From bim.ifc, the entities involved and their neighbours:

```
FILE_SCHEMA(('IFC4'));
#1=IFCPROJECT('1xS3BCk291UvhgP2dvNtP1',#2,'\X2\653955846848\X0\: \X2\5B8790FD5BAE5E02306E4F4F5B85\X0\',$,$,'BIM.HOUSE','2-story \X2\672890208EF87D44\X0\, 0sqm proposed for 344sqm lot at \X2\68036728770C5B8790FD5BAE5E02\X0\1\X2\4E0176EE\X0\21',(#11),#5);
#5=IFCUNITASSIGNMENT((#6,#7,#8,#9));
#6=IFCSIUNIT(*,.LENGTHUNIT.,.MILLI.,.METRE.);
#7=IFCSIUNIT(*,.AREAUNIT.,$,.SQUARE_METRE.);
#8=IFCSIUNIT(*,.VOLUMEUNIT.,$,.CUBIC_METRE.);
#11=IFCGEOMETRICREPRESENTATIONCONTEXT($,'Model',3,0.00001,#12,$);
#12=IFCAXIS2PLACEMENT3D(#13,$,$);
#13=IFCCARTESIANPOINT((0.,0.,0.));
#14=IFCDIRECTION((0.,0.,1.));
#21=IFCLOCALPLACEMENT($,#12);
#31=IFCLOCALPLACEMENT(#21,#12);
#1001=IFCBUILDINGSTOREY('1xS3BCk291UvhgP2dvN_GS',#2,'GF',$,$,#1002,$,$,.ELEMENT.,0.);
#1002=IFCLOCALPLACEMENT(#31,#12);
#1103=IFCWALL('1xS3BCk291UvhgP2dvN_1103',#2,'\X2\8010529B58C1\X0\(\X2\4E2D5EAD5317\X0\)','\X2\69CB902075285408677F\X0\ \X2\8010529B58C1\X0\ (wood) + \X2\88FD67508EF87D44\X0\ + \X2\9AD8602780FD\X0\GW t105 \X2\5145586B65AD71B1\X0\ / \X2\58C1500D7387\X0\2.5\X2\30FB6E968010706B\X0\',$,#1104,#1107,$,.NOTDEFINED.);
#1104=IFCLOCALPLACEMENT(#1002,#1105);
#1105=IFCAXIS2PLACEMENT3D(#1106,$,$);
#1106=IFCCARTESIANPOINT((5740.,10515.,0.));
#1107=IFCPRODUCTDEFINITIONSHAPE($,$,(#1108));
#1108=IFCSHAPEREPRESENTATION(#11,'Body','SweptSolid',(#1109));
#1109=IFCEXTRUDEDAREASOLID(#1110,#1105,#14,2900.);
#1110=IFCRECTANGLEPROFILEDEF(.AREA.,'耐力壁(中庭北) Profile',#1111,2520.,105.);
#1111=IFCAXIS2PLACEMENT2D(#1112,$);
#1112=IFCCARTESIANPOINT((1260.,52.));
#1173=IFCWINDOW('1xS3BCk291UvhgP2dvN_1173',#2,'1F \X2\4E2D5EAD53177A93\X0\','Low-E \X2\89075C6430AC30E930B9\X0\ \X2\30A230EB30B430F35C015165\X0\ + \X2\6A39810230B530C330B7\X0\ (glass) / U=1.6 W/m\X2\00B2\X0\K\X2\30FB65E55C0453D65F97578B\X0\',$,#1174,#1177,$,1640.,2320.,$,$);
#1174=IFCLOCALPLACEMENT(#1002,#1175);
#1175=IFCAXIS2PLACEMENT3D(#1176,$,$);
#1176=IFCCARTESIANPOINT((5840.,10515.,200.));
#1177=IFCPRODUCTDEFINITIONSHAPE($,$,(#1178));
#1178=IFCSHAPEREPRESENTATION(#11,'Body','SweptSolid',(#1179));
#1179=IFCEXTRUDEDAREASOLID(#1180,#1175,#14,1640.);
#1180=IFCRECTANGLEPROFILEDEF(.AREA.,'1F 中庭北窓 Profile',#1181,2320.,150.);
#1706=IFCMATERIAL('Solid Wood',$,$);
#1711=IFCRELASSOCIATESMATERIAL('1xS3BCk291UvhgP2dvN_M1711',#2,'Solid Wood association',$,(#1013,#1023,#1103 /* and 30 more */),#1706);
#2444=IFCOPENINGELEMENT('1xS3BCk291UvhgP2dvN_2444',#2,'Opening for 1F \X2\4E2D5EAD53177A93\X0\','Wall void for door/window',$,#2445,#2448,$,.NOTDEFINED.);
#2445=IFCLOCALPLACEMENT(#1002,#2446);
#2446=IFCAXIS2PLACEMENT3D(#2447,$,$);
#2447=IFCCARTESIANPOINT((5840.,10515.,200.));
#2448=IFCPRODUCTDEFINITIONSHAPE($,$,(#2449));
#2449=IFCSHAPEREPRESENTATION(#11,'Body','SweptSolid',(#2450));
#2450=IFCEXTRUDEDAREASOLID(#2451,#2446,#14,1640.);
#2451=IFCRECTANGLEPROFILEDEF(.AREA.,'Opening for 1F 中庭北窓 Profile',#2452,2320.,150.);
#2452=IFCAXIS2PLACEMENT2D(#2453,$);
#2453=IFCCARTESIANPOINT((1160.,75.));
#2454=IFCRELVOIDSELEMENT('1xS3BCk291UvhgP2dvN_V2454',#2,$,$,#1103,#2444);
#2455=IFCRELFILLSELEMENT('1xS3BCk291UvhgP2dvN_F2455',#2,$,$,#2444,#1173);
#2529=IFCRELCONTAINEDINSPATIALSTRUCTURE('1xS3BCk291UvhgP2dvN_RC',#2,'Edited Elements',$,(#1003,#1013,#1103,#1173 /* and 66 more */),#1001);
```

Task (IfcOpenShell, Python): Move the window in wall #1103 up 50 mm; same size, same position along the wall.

```python
import numpy as np
import ifcopenshell
import ifcopenshell.api.geometry
import ifcopenshell.util.placement
import ifcopenshell.util.unit

model = ifcopenshell.open("bim.ifc")
unit_scale = ifcopenshell.util.unit.calculate_unit_scale(model)

window = model.by_guid("1xS3BCk291UvhgP2dvN_1173")
opening = window.FillsVoids[0].RelatingOpeningElement
dz = 0.05 / unit_scale

shift = np.array([0.0, 0.0, dz])
# The window is not placed relative to its opening, so move both.
for product in (opening, window):
    matrix = ifcopenshell.util.placement.get_local_placement(product.ObjectPlacement)
    matrix[:3, 3] += shift
    ifcopenshell.api.geometry.edit_object_placement(model, product=product, matrix=matrix, is_si=False)

print(f"moved by {dz * unit_scale:+.3f} m")

model.write("bim_edited.ifc")
```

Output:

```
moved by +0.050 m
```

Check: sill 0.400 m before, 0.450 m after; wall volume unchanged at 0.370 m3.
